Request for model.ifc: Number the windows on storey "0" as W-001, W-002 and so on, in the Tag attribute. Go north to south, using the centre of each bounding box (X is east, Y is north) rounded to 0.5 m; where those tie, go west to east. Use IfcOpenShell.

First a look at what the model holds.

```python
import ifcopenshell
import ifcopenshell.util.element
import ifcopenshell.util.placement

model = ifcopenshell.open("model.ifc")
print(model.schema)
storey = next(s for s in model.by_type("IfcBuildingStorey") if s.Name == "0")
windows = [e for e in ifcopenshell.util.element.get_decomposition(storey) if e.is_a("IfcWindow")]
for e in sorted(windows, key=lambda e: e.id()):
    origin = ifcopenshell.util.placement.get_local_placement(e.ObjectPlacement)[:3, 3]
    print(e.id(), e.Tag, e.Name, origin.round(2) + 0.0, sep=" | ")
```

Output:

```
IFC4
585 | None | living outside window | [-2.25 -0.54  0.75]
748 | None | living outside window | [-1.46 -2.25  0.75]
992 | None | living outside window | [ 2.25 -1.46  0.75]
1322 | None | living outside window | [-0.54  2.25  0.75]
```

```python
import ifcopenshell
import ifcopenshell.geom
import ifcopenshell.util.element
import ifcopenshell.util.shape

model = ifcopenshell.open("model.ifc")
settings = ifcopenshell.geom.settings()
settings.set("use-world-coords", True)


def centre(element):
    shape = ifcopenshell.geom.create_shape(settings, element)
    return ifcopenshell.util.shape.get_bbox_centroid(shape.geometry)


storey = next(s for s in model.by_type("IfcBuildingStorey") if s.Name == "0")
windows = [e for e in ifcopenshell.util.element.get_decomposition(storey) if e.is_a("IfcWindow")]

# Insertion points can sit at a corner or the storey origin, so sort by the geometry (in metres).
centres = {e: centre(e) for e in windows}
windows.sort(key=lambda e: (-round(centres[e][1] / 0.5), centres[e][0]))

for i, e in enumerate(windows, start=1):
    number = f"W-0{i:02d}"
    e.Tag = number
    print(e.id(), number)

model.write("model-out.ifc")
```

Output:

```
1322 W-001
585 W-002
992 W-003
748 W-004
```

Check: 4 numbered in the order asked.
